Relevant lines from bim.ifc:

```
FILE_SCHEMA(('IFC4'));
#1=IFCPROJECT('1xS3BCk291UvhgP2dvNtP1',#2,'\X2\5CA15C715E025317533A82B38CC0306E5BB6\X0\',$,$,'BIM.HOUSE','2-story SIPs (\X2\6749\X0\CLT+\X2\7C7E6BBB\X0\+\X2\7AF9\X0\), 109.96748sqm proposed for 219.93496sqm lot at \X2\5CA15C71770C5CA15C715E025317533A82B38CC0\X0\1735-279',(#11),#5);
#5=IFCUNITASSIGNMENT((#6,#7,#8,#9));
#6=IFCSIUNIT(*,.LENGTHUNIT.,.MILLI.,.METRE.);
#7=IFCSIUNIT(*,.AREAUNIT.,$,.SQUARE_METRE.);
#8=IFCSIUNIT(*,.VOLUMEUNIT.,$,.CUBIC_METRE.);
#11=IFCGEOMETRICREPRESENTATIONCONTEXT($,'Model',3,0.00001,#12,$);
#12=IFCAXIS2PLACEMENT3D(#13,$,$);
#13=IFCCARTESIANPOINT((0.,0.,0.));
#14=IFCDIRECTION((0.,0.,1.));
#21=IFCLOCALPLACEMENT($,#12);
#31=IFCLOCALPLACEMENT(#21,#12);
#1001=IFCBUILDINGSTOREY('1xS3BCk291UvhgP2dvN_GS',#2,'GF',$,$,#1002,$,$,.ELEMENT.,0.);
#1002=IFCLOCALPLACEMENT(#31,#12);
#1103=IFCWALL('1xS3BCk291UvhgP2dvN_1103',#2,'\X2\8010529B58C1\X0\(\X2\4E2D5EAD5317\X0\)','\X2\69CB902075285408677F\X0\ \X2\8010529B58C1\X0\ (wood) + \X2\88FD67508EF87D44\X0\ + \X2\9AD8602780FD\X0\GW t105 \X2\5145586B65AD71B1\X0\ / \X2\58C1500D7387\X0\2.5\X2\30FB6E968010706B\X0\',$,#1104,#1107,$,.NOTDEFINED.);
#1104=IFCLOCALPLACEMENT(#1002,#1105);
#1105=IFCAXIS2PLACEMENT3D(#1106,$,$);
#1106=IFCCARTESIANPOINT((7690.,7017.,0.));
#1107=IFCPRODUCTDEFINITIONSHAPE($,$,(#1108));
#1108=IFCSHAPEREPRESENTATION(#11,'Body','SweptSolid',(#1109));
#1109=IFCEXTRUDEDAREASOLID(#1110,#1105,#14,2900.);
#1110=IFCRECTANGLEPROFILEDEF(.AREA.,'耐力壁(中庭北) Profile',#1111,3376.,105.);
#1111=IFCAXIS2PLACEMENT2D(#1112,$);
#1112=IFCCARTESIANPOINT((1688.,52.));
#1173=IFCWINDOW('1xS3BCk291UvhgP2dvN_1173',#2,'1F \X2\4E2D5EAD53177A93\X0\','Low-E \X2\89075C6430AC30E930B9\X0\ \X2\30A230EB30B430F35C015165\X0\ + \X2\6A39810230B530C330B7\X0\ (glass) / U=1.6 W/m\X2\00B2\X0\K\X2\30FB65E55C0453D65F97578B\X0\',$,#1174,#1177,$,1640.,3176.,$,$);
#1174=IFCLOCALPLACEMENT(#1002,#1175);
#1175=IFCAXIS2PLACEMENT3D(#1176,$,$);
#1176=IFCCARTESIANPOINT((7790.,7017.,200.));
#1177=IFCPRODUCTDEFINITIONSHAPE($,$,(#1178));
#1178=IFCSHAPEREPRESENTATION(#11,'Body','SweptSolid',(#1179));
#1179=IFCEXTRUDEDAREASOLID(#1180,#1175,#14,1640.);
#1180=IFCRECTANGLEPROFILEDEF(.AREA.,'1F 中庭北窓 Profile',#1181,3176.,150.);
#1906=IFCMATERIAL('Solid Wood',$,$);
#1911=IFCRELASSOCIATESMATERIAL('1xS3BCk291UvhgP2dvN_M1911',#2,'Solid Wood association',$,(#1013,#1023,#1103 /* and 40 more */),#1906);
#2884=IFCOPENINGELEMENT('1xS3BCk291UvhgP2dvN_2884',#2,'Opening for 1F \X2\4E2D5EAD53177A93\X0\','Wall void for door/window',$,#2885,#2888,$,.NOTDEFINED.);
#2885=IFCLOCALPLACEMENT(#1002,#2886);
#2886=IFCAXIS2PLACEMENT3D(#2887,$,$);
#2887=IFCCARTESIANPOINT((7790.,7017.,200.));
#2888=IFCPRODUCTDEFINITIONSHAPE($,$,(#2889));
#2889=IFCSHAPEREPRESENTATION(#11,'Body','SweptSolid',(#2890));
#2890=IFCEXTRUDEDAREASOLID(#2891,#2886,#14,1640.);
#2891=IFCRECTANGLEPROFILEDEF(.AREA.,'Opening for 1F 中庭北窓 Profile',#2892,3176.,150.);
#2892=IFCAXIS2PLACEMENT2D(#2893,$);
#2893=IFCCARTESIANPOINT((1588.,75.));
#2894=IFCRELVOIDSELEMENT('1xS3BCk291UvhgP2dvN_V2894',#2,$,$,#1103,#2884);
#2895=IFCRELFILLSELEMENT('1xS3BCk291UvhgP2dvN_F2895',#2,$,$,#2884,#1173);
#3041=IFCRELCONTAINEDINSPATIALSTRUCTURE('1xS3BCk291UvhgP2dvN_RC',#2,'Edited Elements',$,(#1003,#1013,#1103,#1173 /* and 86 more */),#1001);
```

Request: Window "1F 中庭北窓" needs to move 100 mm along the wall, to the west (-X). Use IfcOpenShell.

```python
import ifcopenshell
import ifcopenshell.api.geometry
import ifcopenshell.util.placement

model = ifcopenshell.open("bim.ifc")

window = model.by_guid("1xS3BCk291UvhgP2dvN_1173")
opening = window.FillsVoids[0].RelatingOpeningElement
wall = opening.VoidsElements[0].RelatingBuildingElement

wall_matrix = ifcopenshell.util.placement.get_local_placement(wall.ObjectPlacement)
shift = wall_matrix[:3, 0] * -100.0
before = ifcopenshell.util.placement.get_local_placement(window.ObjectPlacement)[:3, 3].copy()

# The window is not placed relative to its opening, so move both.
for product in (opening, window):
    matrix = ifcopenshell.util.placement.get_local_placement(product.ObjectPlacement)
    matrix[:3, 3] += shift
    ifcopenshell.api.geometry.edit_object_placement(model, product=product, matrix=matrix, is_si=False)

after = ifcopenshell.util.placement.get_local_placement(window.ObjectPlacement)[:3, 3]
print("window moved by", (after - before).round(3) + 0.0)

model.write("bim_edited.ifc")
```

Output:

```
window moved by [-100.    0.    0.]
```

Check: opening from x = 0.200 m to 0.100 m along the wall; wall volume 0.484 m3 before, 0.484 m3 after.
